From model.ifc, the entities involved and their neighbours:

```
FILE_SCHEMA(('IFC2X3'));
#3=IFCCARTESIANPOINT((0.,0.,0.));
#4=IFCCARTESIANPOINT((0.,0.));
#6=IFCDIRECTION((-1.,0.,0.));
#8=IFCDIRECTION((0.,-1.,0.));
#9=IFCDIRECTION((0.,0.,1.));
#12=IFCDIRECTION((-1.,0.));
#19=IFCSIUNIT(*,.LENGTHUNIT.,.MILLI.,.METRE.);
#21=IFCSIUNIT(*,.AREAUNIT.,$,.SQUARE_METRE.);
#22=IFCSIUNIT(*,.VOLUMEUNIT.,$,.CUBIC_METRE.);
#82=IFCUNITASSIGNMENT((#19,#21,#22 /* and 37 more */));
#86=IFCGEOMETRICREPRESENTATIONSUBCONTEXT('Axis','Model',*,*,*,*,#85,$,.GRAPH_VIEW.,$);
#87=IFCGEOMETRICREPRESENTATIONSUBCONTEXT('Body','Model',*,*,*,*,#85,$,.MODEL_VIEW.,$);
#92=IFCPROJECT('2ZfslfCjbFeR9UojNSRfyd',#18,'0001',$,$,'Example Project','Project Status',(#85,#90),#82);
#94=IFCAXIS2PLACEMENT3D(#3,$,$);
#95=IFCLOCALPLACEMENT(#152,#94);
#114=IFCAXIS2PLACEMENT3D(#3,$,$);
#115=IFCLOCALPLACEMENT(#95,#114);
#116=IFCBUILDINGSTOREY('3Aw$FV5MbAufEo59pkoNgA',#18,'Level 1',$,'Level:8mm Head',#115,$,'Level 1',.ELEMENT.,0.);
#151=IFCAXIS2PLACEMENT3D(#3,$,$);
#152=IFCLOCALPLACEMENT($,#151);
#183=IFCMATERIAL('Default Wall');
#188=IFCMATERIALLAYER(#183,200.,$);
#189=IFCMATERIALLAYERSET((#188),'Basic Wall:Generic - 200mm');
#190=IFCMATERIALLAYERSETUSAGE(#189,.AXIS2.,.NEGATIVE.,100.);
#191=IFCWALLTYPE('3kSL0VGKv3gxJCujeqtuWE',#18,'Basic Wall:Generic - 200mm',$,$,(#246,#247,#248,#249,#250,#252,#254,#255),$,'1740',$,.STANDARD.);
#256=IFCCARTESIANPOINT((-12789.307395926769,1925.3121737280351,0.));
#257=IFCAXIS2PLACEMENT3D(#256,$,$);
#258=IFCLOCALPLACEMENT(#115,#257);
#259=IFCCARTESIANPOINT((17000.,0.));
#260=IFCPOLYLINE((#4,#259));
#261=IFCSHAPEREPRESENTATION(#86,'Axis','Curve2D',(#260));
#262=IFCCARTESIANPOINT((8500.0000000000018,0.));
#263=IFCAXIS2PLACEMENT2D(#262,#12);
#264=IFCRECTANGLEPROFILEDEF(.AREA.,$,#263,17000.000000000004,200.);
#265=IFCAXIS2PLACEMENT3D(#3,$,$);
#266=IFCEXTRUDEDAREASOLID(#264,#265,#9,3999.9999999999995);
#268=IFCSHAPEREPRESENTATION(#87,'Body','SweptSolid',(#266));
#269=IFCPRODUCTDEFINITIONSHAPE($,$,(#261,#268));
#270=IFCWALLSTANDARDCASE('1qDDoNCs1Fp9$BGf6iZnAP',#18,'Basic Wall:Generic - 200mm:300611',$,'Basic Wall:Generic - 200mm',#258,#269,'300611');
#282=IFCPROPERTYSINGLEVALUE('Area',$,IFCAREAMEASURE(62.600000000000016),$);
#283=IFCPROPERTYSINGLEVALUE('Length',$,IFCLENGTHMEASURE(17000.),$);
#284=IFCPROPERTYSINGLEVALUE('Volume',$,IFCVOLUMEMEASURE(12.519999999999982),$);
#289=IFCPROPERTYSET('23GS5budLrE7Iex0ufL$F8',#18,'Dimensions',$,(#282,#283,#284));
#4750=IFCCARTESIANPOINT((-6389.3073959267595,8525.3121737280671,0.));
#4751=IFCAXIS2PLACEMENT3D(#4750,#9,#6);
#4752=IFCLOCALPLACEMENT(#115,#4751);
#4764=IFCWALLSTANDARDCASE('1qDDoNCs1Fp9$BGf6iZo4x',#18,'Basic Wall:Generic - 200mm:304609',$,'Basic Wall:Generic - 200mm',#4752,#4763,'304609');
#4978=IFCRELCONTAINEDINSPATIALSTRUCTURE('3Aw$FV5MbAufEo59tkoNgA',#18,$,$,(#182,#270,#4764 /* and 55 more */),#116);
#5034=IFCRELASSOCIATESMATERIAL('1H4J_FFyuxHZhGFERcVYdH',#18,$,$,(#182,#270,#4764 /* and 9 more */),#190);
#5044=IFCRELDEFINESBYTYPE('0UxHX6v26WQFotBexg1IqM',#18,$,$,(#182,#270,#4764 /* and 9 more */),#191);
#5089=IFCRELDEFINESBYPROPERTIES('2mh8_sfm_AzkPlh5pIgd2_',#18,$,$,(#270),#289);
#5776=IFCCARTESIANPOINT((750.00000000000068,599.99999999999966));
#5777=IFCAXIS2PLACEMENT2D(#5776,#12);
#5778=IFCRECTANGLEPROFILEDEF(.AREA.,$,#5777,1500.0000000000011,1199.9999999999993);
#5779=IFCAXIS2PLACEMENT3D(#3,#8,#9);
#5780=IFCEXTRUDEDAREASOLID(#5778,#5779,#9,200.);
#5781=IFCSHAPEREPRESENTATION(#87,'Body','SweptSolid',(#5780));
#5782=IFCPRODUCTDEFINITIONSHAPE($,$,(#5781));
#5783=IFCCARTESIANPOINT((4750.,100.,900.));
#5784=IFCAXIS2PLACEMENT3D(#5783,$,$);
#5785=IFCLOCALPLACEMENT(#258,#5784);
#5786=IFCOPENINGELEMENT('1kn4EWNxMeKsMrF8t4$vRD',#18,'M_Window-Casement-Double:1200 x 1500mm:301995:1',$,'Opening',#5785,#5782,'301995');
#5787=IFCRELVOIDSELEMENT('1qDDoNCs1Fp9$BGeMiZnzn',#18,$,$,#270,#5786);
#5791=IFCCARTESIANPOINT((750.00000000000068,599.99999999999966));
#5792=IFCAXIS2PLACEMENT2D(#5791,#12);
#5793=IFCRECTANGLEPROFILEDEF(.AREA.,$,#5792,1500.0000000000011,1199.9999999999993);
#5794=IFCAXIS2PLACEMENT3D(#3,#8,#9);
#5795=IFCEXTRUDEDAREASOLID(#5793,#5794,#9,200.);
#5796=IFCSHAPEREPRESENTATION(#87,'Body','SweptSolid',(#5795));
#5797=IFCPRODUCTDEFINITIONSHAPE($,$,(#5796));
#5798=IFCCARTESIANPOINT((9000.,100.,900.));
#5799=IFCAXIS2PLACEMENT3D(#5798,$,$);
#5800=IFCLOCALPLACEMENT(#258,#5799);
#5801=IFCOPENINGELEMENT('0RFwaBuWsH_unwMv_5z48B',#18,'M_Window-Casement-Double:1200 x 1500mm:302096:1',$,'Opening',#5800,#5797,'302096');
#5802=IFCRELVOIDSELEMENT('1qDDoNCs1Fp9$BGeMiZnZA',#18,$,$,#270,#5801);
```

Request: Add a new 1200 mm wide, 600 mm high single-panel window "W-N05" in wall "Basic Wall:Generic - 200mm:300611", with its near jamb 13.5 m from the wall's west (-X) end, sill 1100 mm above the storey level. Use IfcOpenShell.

```python
import numpy as np
import ifcopenshell
import ifcopenshell.api.feature
import ifcopenshell.api.geometry
import ifcopenshell.api.pset
import ifcopenshell.api.root
import ifcopenshell.api.spatial
import ifcopenshell.api.type
import ifcopenshell.geom
import ifcopenshell.util.element
import ifcopenshell.util.placement
import ifcopenshell.util.representation
import ifcopenshell.util.shape
import ifcopenshell.util.unit

model = ifcopenshell.open("model.ifc")
unit_scale = ifcopenshell.util.unit.calculate_unit_scale(model)
area_scale = ifcopenshell.util.unit.calculate_unit_scale(model, "AREAUNIT")
volume_scale = ifcopenshell.util.unit.calculate_unit_scale(model, "VOLUMEUNIT")
settings = ifcopenshell.geom.settings()


def volume(element):
    """Net volume in cubic metres, openings subtracted."""
    shape = ifcopenshell.geom.create_shape(settings, element)
    return ifcopenshell.util.shape.get_volume(shape.geometry)


wall = model.by_guid("1qDDoNCs1Fp9$BGf6iZnAP")
storey = ifcopenshell.util.element.get_container(wall, ifc_class="IfcBuildingStorey")
context = ifcopenshell.util.representation.get_context(model, "Model", "Body", "MODEL_VIEW")
before = volume(wall)

width, height, from_end, sill = 1.2, 0.6, 13.5, 1.1  # metres

# The wall runs along its own X axis, and the end named is its -X end.
wall_shape = ifcopenshell.geom.create_shape(settings, wall)
x, y, z = ifcopenshell.util.shape.get_vertices(wall_shape.geometry).T
start = x.min() + from_end
face, thickness = float(y.min()), float(y.max() - y.min())
wall_matrix = ifcopenshell.util.placement.get_local_placement(wall.ObjectPlacement)
level = ifcopenshell.util.placement.get_local_placement(storey.ObjectPlacement)[2, 3]


def in_wall(x, y):
    """Placement at x, y metres in the wall's axes, at sill height."""
    matrix = wall_matrix.copy()
    matrix[:, 3] = wall_matrix @ np.array([x / unit_scale, y / unit_scale, 0.0, 1.0])
    matrix[2, 3] = level + sill / unit_scale
    return matrix


# Opening: a box that overshoots both wall faces by 50 mm.
opening = ifcopenshell.api.root.create_entity(model, ifc_class="IfcOpeningElement")
box = ifcopenshell.api.geometry.add_wall_representation(
    model, context=context, length=width, height=height, thickness=thickness + 0.1
)
ifcopenshell.api.geometry.assign_representation(model, product=opening, representation=box)
ifcopenshell.api.geometry.edit_object_placement(model, product=opening, matrix=in_wall(start, face - 0.05), is_si=False)
ifcopenshell.api.feature.add_feature(model, feature=opening, element=wall)

window = ifcopenshell.api.root.create_entity(model, ifc_class="IfcWindow", name="W-N05")
window.OverallWidth, window.OverallHeight = width / unit_scale, height / unit_scale
body = ifcopenshell.api.geometry.add_window_representation(
    model,
    context=context,
    overall_width=window.OverallWidth,
    overall_height=window.OverallHeight,
    partition_type="SINGLE_PANEL",
)
ifcopenshell.api.geometry.assign_representation(model, product=window, representation=body)
ifcopenshell.api.spatial.assign_container(model, products=[window], relating_structure=storey)
fills = ifcopenshell.api.feature.add_filling(model, opening=opening, element=window)
fills.OwnerHistory = window.OwnerHistory  # required in IFC2X3

# IFC2X3 keeps the operation on the window style.
style = ifcopenshell.api.root.create_entity(model, ifc_class="IfcWindowStyle", name="W-N05")
style.OperationType, style.ConstructionType = "SINGLE_PANEL", "NOTDEFINED"
style.ParameterTakesPrecedence = style.Sizeable = False
ifcopenshell.api.type.assign_type(model, related_objects=[window], relating_type=style)

# Centre the window in the wall's thickness.
ifcopenshell.api.geometry.edit_object_placement(model, product=window, matrix=in_wall(start, face), is_si=False)
window_shape = ifcopenshell.geom.create_shape(settings, window)
depth = ifcopenshell.util.shape.get_vertices(window_shape.geometry)[:, 1]
offset = face + thickness / 2 - (depth.min() + depth.max()) / 2
ifcopenshell.api.geometry.edit_object_placement(model, product=window, matrix=in_wall(start, offset), is_si=False)

after = volume(wall)

# Update the wall's stored quantities.
pset = model.by_id(ifcopenshell.util.element.get_pset(wall, "Dimensions", should_inherit=False)["id"])
ifcopenshell.api.pset.edit_pset(model, pset=pset, properties={
    "Area": model.create_entity("IfcAreaMeasure", after / thickness / area_scale),
    "Volume": model.create_entity("IfcVolumeMeasure", after / volume_scale),
})

print(f"wall volume {before:.3f} -> {after:.3f} m3")

model.write("model_updated.ifc")
```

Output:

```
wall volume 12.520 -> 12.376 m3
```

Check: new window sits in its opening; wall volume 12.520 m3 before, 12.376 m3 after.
